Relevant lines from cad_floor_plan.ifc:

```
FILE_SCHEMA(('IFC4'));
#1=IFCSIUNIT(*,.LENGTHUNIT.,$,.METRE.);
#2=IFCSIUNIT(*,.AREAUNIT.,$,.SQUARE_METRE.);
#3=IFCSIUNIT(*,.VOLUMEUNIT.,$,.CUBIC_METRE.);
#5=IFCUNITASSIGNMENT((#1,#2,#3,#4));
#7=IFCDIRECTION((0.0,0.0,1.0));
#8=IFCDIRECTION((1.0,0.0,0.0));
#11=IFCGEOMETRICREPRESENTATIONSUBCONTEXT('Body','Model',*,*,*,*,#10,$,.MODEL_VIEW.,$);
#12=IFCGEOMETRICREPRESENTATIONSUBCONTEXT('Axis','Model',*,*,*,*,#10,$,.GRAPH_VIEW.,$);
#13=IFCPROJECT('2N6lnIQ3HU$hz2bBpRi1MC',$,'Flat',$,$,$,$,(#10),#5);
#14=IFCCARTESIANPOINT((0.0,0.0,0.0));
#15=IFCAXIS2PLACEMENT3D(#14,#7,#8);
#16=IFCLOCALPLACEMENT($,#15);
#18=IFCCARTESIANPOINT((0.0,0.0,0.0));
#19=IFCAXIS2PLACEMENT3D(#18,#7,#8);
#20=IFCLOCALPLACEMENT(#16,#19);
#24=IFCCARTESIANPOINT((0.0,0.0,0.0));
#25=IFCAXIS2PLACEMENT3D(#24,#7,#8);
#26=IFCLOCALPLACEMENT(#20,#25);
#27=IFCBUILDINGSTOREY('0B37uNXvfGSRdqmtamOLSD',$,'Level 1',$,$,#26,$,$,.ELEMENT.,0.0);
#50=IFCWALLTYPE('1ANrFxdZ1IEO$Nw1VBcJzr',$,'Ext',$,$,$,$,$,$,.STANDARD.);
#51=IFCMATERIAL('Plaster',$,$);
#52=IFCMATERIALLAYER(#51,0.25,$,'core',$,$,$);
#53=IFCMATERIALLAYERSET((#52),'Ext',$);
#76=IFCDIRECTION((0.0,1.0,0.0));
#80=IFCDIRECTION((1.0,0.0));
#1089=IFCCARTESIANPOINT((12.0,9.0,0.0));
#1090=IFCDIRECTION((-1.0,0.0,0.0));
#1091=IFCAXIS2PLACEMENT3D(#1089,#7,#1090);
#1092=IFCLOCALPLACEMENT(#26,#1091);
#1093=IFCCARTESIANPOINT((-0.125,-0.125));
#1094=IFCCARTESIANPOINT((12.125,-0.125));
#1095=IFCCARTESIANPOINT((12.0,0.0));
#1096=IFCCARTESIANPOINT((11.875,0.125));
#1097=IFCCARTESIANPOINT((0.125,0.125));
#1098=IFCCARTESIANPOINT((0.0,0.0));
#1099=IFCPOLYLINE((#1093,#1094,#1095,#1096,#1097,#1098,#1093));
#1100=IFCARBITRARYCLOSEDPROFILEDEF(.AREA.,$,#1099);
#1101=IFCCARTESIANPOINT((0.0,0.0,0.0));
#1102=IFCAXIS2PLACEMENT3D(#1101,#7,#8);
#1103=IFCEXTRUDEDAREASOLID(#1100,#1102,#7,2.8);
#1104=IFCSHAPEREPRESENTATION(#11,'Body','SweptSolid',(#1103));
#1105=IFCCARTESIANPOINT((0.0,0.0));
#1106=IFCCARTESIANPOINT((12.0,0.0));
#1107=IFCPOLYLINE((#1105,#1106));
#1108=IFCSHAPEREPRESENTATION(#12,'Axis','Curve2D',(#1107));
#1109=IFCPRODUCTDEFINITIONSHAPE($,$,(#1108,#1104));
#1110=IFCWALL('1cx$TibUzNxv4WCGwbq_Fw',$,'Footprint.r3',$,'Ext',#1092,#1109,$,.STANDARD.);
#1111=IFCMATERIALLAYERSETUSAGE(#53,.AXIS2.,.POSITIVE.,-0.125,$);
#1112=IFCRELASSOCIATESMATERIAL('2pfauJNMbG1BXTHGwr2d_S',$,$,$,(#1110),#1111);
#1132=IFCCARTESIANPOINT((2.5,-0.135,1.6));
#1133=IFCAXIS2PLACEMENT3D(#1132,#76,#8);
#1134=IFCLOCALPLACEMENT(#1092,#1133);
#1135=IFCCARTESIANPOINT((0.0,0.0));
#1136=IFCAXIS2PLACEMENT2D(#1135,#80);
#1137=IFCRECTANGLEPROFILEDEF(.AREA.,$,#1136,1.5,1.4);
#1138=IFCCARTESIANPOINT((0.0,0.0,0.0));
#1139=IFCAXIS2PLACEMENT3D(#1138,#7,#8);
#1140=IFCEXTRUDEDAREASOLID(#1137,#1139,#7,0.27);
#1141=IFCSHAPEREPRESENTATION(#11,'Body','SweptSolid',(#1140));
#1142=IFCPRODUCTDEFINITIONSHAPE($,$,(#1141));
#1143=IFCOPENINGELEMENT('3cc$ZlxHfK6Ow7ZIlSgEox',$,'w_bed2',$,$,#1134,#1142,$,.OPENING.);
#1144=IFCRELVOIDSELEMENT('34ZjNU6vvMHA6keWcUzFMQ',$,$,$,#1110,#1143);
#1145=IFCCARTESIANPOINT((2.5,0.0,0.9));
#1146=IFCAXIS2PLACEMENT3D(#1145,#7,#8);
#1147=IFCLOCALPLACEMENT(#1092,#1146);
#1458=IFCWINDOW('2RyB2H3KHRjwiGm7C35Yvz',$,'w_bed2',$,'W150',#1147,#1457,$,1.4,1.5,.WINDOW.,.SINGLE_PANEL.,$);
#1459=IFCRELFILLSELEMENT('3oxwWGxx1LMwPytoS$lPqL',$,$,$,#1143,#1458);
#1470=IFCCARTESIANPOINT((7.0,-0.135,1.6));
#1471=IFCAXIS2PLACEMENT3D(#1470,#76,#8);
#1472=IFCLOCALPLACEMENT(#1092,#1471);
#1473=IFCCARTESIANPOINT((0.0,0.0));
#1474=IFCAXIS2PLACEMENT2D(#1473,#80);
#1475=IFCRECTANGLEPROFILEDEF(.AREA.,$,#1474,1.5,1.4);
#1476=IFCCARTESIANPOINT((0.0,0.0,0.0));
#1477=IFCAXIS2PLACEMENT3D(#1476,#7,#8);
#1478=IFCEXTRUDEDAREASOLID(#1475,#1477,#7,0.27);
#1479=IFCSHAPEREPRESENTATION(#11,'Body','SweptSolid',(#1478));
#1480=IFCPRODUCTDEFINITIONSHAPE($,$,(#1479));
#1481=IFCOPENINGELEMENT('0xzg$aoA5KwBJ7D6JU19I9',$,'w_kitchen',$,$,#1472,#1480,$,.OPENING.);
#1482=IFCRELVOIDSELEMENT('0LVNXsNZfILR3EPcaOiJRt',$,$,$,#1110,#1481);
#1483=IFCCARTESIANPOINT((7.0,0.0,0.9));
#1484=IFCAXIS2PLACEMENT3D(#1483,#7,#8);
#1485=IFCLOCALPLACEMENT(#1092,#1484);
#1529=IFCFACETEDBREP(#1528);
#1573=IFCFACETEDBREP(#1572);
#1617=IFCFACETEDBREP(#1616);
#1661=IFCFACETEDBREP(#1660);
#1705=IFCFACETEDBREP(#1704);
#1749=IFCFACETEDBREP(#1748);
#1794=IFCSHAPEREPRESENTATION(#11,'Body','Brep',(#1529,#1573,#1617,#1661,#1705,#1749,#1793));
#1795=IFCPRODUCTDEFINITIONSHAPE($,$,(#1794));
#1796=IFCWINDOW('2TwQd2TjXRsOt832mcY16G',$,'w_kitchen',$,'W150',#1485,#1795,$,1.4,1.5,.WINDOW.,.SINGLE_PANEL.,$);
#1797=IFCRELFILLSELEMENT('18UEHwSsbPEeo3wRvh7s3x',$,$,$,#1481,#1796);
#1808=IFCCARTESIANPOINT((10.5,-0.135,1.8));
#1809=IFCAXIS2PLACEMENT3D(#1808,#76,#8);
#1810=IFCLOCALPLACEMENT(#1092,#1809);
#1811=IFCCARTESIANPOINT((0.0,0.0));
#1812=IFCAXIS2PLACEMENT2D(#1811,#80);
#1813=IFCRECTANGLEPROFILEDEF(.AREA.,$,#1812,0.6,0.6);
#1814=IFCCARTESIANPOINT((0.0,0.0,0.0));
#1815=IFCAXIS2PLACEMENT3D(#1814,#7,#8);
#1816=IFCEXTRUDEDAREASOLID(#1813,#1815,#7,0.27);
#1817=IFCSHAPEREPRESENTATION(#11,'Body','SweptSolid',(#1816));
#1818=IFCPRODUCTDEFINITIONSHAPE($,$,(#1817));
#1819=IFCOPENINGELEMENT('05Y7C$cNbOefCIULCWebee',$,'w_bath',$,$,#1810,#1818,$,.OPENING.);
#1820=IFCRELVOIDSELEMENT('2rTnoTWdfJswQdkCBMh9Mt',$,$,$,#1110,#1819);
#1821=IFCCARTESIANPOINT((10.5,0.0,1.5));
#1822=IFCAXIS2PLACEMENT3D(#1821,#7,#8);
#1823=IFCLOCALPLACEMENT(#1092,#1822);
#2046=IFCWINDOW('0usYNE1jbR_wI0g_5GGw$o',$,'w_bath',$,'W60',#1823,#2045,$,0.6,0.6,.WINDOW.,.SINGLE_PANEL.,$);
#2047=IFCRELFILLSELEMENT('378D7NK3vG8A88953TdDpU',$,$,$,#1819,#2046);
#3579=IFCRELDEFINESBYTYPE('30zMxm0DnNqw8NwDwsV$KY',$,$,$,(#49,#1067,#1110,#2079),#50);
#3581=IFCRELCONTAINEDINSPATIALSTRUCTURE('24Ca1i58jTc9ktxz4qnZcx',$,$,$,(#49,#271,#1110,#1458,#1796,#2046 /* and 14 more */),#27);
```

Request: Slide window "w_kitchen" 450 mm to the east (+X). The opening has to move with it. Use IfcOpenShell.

```python
import ifcopenshell
import ifcopenshell.api.geometry
import ifcopenshell.util.placement

model = ifcopenshell.open("cad_floor_plan.ifc")

window = model.by_guid("2TwQd2TjXRsOt832mcY16G")
opening = window.FillsVoids[0].RelatingOpeningElement
wall = opening.VoidsElements[0].RelatingBuildingElement

wall_matrix = ifcopenshell.util.placement.get_local_placement(wall.ObjectPlacement)
shift = wall_matrix[:3, 0] * -0.45
before = ifcopenshell.util.placement.get_local_placement(window.ObjectPlacement)[:3, 3].copy()

# The window is not placed relative to its opening, so move both.
for product in (opening, window):
    matrix = ifcopenshell.util.placement.get_local_placement(product.ObjectPlacement)
    matrix[:3, 3] += shift
    ifcopenshell.api.geometry.edit_object_placement(model, product=product, matrix=matrix, is_si=False)

after = ifcopenshell.util.placement.get_local_placement(window.ObjectPlacement)[:3, 3]
print("window moved by", (after - before).round(3) + 0.0)

model.write("cad_floor_plan_v2.ifc")
```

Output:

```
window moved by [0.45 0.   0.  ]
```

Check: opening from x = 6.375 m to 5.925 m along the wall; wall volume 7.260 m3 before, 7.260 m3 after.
